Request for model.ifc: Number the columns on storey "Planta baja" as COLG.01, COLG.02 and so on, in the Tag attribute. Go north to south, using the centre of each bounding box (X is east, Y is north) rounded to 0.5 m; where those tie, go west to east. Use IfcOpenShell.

First a look at what the model holds.

```python
import ifcopenshell
import ifcopenshell.util.element
import ifcopenshell.util.placement

model = ifcopenshell.open("model.ifc")
print(model.schema)
storey = next(s for s in model.by_type("IfcBuildingStorey") if s.Name == "Planta baja")
columns = [e for e in ifcopenshell.util.element.get_decomposition(storey) if e.is_a("IfcColumn")]
for e in sorted(columns, key=lambda e: e.id()):
    origin = ifcopenshell.util.placement.get_local_placement(e.ObjectPlacement)[:3, 3]
    print(e.id(), e.Tag, e.Name, origin.round(2) + 0.0, sep=" | ")
```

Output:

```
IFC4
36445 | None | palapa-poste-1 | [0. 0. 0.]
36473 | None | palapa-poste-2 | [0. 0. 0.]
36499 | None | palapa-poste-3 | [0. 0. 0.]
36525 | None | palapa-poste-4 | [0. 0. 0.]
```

```python
import ifcopenshell
import ifcopenshell.geom
import ifcopenshell.util.element
import ifcopenshell.util.shape

model = ifcopenshell.open("model.ifc")
settings = ifcopenshell.geom.settings()
settings.set("use-world-coords", True)


def centre(element):
    shape = ifcopenshell.geom.create_shape(settings, element)
    return ifcopenshell.util.shape.get_bbox_centroid(shape.geometry)


storey = next(s for s in model.by_type("IfcBuildingStorey") if s.Name == "Planta baja")
columns = [e for e in ifcopenshell.util.element.get_decomposition(storey) if e.is_a("IfcColumn")]

# Insertion points can sit at a corner or the storey origin, so sort by the geometry (in metres).
centres = {e: centre(e) for e in columns}
columns.sort(key=lambda e: (-round(centres[e][1] / 0.5), centres[e][0]))

for i, e in enumerate(columns, start=1):
    number = f"COLG.{i:02d}"
    e.Tag = number
    print(e.id(), number)

model.write("model_edited.ifc")
```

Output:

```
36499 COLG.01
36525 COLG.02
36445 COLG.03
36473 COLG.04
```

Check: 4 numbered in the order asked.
